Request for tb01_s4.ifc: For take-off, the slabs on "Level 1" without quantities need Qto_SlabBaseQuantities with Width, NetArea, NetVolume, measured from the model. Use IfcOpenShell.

First a look at what the model holds.

```python
import ifcopenshell
import ifcopenshell.util.element
import ifcopenshell.util.unit

model = ifcopenshell.open("tb01_s4.ifc")
print(model.schema)
for unit_type in ("LENGTHUNIT", "AREAUNIT", "VOLUMEUNIT"):
    print(unit_type, ifcopenshell.util.unit.calculate_unit_scale(model, unit_type))
storey = next(s for s in model.by_type("IfcBuildingStorey") if s.Name == "Level 1")
slabs = [e for e in ifcopenshell.util.element.get_decomposition(storey) if e.is_a("IfcSlab")]
for e in sorted(slabs, key=lambda e: e.id()):
    print(e.id(), e.is_a(), e.Name, list(ifcopenshell.util.element.get_psets(e, qtos_only=True)), sep=" | ")
```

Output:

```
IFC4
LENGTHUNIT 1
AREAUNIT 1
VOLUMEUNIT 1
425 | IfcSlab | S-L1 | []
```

```python
import ifcopenshell
import ifcopenshell.api.pset
import ifcopenshell.geom
import ifcopenshell.util.element
import ifcopenshell.util.shape
import ifcopenshell.util.unit

model = ifcopenshell.open("tb01_s4.ifc")
unit_scale = ifcopenshell.util.unit.calculate_unit_scale(model)
area_scale = ifcopenshell.util.unit.calculate_unit_scale(model, "AREAUNIT")
volume_scale = ifcopenshell.util.unit.calculate_unit_scale(model, "VOLUMEUNIT")
settings = ifcopenshell.geom.settings()

storey = next(s for s in model.by_type("IfcBuildingStorey") if s.Name == "Level 1")
slabs = [e for e in ifcopenshell.util.element.get_decomposition(storey) if e.is_a("IfcSlab")]

for e in sorted(slabs, key=lambda e: e.id()):
    if ifcopenshell.util.element.get_psets(e, qtos_only=True, should_inherit=False):
        continue
    # Geometry comes back in metres, in the element's own axes.
    shape = ifcopenshell.geom.create_shape(settings, e)
    values = {
        "Width": ifcopenshell.util.shape.get_z(shape.geometry) / unit_scale,
        "NetArea": ifcopenshell.util.shape.get_footprint_area(shape.geometry) / area_scale,
        "NetVolume": ifcopenshell.util.shape.get_volume(shape.geometry) / volume_scale,
    }
    qto = ifcopenshell.api.pset.add_qto(model, product=e, name="Qto_SlabBaseQuantities")
    ifcopenshell.api.pset.edit_qto(model, qto=qto, properties=values)
    print(e.id(), {k: round(v, 3) for k, v in values.items()})

model.write("tb01_s4-out.ifc")
```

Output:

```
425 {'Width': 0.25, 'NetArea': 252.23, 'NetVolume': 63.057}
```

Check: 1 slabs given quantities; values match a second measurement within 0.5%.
